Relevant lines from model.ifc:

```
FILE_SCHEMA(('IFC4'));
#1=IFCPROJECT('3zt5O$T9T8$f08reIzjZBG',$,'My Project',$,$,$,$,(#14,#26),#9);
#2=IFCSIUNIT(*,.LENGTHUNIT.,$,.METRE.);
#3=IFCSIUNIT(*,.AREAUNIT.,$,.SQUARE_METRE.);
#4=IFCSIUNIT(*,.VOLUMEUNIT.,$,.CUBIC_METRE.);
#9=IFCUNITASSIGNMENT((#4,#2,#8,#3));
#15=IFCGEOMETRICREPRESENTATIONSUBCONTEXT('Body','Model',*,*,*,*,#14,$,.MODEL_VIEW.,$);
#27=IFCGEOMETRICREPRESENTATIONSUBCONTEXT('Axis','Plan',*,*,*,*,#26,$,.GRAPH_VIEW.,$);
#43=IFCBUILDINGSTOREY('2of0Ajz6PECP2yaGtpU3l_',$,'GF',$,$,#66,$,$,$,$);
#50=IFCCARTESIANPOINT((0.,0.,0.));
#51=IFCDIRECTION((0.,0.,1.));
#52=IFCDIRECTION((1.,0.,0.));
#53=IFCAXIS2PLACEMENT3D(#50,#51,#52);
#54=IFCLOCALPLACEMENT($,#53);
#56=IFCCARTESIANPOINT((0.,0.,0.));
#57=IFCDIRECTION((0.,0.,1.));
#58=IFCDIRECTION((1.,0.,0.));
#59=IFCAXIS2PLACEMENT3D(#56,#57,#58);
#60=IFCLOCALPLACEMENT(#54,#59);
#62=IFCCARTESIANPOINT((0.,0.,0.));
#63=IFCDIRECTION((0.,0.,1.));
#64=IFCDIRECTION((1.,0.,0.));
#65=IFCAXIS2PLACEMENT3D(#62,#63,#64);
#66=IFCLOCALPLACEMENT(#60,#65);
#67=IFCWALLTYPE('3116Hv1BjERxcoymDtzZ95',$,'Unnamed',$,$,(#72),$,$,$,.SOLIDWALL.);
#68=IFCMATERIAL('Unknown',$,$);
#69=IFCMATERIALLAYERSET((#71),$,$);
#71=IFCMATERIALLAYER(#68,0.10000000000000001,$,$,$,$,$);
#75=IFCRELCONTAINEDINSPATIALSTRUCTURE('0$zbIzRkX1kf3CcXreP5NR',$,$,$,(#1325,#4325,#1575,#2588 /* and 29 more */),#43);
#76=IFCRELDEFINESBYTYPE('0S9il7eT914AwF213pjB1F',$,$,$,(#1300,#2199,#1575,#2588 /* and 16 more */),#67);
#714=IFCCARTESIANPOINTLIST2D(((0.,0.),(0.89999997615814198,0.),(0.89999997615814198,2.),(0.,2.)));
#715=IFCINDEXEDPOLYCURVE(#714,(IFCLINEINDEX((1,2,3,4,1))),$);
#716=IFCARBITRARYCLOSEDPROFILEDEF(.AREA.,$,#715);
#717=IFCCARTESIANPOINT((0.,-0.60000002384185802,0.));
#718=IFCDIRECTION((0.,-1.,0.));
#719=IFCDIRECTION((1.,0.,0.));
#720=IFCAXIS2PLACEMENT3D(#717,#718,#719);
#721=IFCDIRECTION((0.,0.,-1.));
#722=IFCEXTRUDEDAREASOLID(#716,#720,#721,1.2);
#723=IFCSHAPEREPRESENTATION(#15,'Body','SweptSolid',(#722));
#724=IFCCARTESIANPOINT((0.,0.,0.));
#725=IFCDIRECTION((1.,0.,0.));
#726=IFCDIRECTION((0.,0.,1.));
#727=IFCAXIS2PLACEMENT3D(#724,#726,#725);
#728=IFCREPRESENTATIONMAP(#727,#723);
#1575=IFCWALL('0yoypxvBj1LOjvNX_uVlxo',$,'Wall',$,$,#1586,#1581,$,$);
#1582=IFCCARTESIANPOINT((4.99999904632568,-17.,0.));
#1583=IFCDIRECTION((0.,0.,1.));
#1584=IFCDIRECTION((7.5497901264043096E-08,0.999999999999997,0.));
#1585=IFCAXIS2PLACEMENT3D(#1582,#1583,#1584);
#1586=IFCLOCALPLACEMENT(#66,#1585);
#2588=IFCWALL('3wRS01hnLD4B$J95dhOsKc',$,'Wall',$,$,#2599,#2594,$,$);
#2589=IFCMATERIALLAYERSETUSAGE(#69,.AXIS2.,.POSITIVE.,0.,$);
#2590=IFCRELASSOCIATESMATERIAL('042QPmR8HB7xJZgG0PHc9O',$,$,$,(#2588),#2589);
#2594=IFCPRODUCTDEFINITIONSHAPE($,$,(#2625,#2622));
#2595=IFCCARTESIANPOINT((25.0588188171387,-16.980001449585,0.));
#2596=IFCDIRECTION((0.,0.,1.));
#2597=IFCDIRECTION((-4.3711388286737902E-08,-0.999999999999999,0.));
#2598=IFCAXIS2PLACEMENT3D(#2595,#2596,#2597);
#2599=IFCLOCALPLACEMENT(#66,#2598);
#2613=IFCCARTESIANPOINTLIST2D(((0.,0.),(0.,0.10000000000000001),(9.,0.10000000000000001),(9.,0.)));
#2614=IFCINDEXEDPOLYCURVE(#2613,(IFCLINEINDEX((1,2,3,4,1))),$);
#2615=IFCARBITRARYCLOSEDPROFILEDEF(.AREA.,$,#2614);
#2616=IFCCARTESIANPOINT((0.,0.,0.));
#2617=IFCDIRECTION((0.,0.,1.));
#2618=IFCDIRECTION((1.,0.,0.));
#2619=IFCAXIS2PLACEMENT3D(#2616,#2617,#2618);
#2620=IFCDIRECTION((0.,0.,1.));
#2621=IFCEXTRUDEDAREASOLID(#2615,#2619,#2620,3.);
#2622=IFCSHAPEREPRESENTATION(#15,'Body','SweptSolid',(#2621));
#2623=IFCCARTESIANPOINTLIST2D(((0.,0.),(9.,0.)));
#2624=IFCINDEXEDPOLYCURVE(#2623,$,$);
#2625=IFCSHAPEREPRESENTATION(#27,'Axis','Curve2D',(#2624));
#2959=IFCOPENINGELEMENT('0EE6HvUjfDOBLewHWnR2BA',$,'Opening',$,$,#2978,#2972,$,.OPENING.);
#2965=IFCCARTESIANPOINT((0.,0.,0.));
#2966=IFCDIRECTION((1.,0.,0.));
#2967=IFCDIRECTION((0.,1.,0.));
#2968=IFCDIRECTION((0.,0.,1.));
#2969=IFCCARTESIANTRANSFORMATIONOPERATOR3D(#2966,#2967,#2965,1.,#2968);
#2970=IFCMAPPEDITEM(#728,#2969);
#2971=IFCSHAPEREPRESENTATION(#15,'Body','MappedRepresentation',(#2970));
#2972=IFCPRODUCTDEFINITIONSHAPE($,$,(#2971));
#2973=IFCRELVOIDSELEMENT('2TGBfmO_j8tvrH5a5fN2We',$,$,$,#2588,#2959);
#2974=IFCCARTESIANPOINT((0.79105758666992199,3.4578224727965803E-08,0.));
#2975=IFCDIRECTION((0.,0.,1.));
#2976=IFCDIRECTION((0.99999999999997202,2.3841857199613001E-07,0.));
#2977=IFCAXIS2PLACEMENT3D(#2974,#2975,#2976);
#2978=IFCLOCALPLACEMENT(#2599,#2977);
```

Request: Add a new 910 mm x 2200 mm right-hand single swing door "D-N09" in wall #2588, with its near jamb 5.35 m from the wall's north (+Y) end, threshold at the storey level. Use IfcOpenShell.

```python
import numpy as np
import ifcopenshell
import ifcopenshell.api.feature
import ifcopenshell.api.geometry
import ifcopenshell.api.root
import ifcopenshell.api.spatial
import ifcopenshell.geom
import ifcopenshell.util.element
import ifcopenshell.util.placement
import ifcopenshell.util.representation
import ifcopenshell.util.shape
import ifcopenshell.util.unit

model = ifcopenshell.open("model.ifc")
unit_scale = ifcopenshell.util.unit.calculate_unit_scale(model)
settings = ifcopenshell.geom.settings()


def volume(element):
    """Net volume in cubic metres, openings subtracted."""
    shape = ifcopenshell.geom.create_shape(settings, element)
    return ifcopenshell.util.shape.get_volume(shape.geometry)


wall = model.by_guid("3wRS01hnLD4B$J95dhOsKc")
storey = ifcopenshell.util.element.get_container(wall, ifc_class="IfcBuildingStorey")
context = ifcopenshell.util.representation.get_context(model, "Model", "Body", "MODEL_VIEW")
before = volume(wall)

width, height, from_end, sill = 0.91, 2.2, 5.35, 0.0  # metres

# The wall runs along its own X axis, and the end named is its -X end.
wall_shape = ifcopenshell.geom.create_shape(settings, wall)
x, y, z = ifcopenshell.util.shape.get_vertices(wall_shape.geometry).T
start = x.min() + from_end
face, thickness = float(y.min()), float(y.max() - y.min())
wall_matrix = ifcopenshell.util.placement.get_local_placement(wall.ObjectPlacement)
level = ifcopenshell.util.placement.get_local_placement(storey.ObjectPlacement)[2, 3]


def in_wall(x, y):
    """Placement at x, y metres in the wall's axes, at sill height."""
    matrix = wall_matrix.copy()
    matrix[:, 3] = wall_matrix @ np.array([x / unit_scale, y / unit_scale, 0.0, 1.0])
    matrix[2, 3] = level + sill / unit_scale
    return matrix


# Opening: a box that overshoots both wall faces by 50 mm.
opening = ifcopenshell.api.root.create_entity(model, ifc_class="IfcOpeningElement", predefined_type="OPENING")
box = ifcopenshell.api.geometry.add_wall_representation(
    model, context=context, length=width, height=height, thickness=thickness + 0.1
)
ifcopenshell.api.geometry.assign_representation(model, product=opening, representation=box)
ifcopenshell.api.geometry.edit_object_placement(model, product=opening, matrix=in_wall(start, face - 0.05), is_si=False)
ifcopenshell.api.feature.add_feature(model, feature=opening, element=wall)

door = ifcopenshell.api.root.create_entity(model, ifc_class="IfcDoor", name="D-N09", predefined_type="DOOR")
door.OverallWidth, door.OverallHeight = width / unit_scale, height / unit_scale
door.OperationType = "SINGLE_SWING_RIGHT"
body = ifcopenshell.api.geometry.add_door_representation(
    model,
    context=context,
    overall_width=door.OverallWidth,
    overall_height=door.OverallHeight,
    operation_type="SINGLE_SWING_RIGHT",
    lining_properties={"LiningDepth": thickness / unit_scale, "ThresholdDepth": thickness / unit_scale},
)
ifcopenshell.api.geometry.assign_representation(model, product=door, representation=body)
ifcopenshell.api.spatial.assign_container(model, products=[door], relating_structure=storey)
ifcopenshell.api.feature.add_filling(model, opening=opening, element=door)

# The lining spans the wall, so the door starts at the wall face.
ifcopenshell.api.geometry.edit_object_placement(model, product=door, matrix=in_wall(start, face), is_si=False)

after = volume(wall)

print(f"wall volume {before:.3f} -> {after:.3f} m3")

model.write("model_edited.ifc")
```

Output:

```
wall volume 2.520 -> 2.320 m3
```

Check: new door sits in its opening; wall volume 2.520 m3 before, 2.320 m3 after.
